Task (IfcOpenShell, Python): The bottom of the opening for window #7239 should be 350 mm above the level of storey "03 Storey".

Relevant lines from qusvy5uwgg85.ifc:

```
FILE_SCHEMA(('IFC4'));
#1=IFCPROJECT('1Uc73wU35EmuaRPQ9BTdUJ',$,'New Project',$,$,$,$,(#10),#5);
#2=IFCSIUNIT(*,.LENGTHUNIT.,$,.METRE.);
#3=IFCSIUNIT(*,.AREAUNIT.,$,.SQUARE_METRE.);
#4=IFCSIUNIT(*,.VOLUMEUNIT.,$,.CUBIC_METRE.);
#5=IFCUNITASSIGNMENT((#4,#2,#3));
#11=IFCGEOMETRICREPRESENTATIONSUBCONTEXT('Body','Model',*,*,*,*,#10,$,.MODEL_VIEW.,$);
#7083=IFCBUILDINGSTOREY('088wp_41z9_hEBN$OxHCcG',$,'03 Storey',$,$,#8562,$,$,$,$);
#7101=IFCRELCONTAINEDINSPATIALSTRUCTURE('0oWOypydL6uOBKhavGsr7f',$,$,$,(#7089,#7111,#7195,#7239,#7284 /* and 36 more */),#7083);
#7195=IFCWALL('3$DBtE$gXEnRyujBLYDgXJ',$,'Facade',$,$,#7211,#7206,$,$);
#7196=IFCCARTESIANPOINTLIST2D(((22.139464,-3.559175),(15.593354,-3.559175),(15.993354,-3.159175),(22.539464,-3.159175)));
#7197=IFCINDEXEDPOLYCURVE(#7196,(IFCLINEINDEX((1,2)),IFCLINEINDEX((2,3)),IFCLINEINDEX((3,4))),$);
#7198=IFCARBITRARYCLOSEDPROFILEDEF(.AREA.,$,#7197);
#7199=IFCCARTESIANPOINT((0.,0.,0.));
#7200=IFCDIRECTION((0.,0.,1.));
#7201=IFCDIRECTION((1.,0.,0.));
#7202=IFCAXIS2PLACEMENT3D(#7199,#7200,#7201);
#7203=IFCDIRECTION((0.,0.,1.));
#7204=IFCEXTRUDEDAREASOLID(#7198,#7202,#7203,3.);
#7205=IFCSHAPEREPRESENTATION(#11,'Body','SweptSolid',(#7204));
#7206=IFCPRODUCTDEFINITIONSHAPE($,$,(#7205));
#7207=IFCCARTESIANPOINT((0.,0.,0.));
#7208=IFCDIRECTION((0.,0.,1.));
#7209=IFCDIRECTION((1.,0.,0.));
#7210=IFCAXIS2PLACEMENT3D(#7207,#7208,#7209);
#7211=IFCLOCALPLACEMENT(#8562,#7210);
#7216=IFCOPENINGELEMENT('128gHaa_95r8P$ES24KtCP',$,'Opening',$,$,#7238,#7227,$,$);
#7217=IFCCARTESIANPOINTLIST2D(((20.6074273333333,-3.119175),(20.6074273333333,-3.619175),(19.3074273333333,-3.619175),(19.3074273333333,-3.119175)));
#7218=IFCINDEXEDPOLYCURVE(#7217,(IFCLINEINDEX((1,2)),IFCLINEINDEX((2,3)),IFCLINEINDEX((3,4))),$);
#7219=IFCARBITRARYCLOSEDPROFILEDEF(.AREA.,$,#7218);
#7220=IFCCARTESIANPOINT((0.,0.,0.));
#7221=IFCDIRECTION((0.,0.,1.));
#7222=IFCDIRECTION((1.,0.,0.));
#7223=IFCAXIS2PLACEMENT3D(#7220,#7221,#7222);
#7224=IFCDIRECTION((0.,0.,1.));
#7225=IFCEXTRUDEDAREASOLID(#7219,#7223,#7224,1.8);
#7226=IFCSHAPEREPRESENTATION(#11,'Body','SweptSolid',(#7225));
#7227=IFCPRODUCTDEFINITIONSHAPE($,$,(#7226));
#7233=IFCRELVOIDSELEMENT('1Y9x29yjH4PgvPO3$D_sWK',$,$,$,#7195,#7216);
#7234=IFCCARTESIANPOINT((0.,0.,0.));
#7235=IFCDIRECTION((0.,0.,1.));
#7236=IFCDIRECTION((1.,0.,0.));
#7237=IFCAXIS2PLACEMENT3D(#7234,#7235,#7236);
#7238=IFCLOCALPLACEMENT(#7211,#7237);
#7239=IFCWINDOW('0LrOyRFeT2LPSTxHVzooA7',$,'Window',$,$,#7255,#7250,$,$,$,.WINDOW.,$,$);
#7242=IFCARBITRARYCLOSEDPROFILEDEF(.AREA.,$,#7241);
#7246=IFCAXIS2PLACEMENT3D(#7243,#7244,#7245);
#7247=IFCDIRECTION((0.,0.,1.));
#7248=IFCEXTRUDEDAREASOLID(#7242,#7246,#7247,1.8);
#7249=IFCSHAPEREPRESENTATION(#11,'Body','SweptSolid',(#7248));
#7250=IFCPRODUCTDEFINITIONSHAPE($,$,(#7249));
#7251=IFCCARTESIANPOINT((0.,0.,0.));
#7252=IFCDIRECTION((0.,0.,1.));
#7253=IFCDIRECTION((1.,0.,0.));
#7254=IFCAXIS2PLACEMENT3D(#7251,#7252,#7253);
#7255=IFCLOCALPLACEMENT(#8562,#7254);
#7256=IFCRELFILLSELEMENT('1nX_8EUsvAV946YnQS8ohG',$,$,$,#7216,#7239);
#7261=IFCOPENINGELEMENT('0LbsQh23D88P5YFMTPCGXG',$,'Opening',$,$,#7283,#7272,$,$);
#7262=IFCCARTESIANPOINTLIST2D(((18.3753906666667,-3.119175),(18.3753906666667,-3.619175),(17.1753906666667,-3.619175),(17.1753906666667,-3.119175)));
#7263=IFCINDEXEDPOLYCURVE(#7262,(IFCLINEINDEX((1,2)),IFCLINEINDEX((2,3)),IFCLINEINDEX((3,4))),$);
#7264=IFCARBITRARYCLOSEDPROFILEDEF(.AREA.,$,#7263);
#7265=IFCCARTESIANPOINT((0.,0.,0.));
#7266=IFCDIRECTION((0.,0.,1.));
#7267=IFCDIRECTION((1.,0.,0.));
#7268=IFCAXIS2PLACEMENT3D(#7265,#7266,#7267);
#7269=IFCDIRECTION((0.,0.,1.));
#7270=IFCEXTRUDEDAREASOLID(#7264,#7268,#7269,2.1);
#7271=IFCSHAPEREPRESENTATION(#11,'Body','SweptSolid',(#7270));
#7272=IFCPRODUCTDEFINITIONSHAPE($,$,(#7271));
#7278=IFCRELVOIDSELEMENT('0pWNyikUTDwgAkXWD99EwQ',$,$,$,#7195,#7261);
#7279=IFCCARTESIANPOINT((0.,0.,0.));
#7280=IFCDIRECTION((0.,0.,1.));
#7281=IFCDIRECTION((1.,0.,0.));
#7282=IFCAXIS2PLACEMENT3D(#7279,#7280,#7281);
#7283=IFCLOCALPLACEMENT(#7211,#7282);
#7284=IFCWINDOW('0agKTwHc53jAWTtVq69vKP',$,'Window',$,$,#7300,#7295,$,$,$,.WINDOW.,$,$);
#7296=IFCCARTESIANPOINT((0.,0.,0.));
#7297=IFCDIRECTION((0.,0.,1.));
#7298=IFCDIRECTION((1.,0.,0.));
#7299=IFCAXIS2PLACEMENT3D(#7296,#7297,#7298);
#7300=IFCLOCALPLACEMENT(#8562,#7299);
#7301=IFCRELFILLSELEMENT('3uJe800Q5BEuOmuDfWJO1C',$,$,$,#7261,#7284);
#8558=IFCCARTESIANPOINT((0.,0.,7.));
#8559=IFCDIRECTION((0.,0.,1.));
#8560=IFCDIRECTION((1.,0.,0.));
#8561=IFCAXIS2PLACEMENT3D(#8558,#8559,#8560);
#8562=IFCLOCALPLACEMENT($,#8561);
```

```python
import numpy as np
import ifcopenshell
import ifcopenshell.api.geometry
import ifcopenshell.geom
import ifcopenshell.util.element
import ifcopenshell.util.placement
import ifcopenshell.util.shape
import ifcopenshell.util.unit

model = ifcopenshell.open("qusvy5uwgg85.ifc")
unit_scale = ifcopenshell.util.unit.calculate_unit_scale(model)

window = model.by_guid("0LrOyRFeT2LPSTxHVzooA7")
opening = window.FillsVoids[0].RelatingOpeningElement
storey = ifcopenshell.util.element.get_container(window, ifc_class="IfcBuildingStorey")
level = ifcopenshell.util.placement.get_local_placement(storey.ObjectPlacement)[2, 3]

# The opening's origin need not be at the sill, so measure its lowest point.
shape = ifcopenshell.geom.create_shape(ifcopenshell.geom.settings(), opening)
bottom = ifcopenshell.util.shape.get_shape_bottom_elevation(shape, shape.geometry) / unit_scale
dz = level + 0.35 - bottom

shift = np.array([0.0, 0.0, dz])
# The window is not placed relative to its opening, so move both.
for product in (opening, window):
    matrix = ifcopenshell.util.placement.get_local_placement(product.ObjectPlacement)
    matrix[:3, 3] += shift
    ifcopenshell.api.geometry.edit_object_placement(model, product=product, matrix=matrix, is_si=False)

print(f"moved by {dz * unit_scale:+.3f} m")

model.write("qusvy5uwgg85-out.ifc")
```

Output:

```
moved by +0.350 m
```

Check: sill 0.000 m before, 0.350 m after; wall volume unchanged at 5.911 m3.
